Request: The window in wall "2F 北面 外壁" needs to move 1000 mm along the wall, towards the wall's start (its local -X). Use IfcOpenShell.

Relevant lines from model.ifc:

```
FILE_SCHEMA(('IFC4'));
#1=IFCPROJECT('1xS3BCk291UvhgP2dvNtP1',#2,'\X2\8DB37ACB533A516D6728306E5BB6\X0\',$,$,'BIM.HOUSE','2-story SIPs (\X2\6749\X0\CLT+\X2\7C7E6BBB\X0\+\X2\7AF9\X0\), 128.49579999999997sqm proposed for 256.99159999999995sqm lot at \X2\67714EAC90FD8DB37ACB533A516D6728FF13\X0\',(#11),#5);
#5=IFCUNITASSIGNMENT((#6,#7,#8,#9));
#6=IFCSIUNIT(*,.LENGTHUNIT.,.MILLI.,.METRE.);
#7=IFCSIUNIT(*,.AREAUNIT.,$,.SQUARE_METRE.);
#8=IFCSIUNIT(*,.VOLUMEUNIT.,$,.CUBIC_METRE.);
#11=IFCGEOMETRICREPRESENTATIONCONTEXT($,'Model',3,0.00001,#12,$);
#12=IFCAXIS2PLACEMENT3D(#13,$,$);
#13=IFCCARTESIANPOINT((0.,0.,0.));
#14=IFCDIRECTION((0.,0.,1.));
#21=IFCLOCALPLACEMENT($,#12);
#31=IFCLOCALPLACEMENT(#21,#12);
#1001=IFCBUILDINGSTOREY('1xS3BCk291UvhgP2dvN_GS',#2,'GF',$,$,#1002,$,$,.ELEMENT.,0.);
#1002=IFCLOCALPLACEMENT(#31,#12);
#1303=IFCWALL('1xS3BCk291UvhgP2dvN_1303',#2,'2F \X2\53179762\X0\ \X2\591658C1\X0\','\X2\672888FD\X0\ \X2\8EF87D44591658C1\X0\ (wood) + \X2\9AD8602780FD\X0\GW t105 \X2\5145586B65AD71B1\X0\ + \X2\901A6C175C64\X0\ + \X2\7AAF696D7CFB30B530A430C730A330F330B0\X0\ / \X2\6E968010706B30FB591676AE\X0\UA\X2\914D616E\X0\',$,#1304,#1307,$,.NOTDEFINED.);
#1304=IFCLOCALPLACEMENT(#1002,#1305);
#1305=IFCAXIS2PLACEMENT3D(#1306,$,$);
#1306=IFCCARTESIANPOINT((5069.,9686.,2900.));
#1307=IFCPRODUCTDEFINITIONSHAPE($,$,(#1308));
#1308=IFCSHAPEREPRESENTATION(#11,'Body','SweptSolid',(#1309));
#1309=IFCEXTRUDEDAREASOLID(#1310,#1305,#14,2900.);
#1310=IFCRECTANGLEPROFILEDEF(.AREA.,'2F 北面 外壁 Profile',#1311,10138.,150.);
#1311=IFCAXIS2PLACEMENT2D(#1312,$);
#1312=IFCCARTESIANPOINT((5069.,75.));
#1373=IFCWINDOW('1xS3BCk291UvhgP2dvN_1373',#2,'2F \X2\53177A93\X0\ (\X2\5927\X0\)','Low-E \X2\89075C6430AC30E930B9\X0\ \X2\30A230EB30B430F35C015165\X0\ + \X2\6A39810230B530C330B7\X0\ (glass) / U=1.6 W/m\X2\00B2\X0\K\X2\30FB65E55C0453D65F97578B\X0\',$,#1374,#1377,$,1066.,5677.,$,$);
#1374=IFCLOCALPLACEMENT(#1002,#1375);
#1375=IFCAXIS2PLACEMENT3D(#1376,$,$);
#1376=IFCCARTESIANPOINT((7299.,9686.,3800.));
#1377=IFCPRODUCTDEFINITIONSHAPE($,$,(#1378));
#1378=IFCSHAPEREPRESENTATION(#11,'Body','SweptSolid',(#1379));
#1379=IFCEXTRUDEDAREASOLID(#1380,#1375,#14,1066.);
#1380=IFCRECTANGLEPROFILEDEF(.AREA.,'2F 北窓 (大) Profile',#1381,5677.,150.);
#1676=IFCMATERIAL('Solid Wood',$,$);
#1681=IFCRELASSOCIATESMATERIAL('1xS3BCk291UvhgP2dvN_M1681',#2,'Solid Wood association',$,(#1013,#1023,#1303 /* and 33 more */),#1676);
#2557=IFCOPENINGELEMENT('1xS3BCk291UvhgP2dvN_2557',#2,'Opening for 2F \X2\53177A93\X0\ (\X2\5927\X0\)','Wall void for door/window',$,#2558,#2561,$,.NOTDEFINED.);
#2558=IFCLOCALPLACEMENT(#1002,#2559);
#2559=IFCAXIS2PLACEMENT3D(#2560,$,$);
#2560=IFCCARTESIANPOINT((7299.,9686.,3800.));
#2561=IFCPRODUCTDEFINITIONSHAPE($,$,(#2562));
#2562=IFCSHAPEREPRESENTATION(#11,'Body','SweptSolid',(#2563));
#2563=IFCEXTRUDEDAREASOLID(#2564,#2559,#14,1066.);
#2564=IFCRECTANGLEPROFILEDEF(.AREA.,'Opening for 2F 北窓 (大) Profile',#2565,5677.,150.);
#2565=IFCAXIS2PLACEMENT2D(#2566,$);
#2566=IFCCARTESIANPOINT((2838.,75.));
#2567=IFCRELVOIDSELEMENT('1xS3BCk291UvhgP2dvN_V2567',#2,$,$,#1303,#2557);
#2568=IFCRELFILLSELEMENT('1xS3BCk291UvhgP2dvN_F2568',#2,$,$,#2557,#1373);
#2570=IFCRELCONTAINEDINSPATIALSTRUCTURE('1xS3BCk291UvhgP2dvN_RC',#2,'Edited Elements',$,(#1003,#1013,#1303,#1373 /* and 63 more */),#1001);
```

```python
import ifcopenshell
import ifcopenshell.api.geometry
import ifcopenshell.util.placement

model = ifcopenshell.open("model.ifc")

window = model.by_guid("1xS3BCk291UvhgP2dvN_1373")
opening = window.FillsVoids[0].RelatingOpeningElement
wall = opening.VoidsElements[0].RelatingBuildingElement

wall_matrix = ifcopenshell.util.placement.get_local_placement(wall.ObjectPlacement)
shift = wall_matrix[:3, 0] * -1000.0
before = ifcopenshell.util.placement.get_local_placement(window.ObjectPlacement)[:3, 3].copy()

# The window is not placed relative to its opening, so move both.
for product in (opening, window):
    matrix = ifcopenshell.util.placement.get_local_placement(product.ObjectPlacement)
    matrix[:3, 3] += shift
    ifcopenshell.api.geometry.edit_object_placement(model, product=product, matrix=matrix, is_si=False)

after = ifcopenshell.util.placement.get_local_placement(window.ObjectPlacement)[:3, 3]
print("window moved by", (after - before).round(3) + 0.0)

model.write("model_edited.ifc")
```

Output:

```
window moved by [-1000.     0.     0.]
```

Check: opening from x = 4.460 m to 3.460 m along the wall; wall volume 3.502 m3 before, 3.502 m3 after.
